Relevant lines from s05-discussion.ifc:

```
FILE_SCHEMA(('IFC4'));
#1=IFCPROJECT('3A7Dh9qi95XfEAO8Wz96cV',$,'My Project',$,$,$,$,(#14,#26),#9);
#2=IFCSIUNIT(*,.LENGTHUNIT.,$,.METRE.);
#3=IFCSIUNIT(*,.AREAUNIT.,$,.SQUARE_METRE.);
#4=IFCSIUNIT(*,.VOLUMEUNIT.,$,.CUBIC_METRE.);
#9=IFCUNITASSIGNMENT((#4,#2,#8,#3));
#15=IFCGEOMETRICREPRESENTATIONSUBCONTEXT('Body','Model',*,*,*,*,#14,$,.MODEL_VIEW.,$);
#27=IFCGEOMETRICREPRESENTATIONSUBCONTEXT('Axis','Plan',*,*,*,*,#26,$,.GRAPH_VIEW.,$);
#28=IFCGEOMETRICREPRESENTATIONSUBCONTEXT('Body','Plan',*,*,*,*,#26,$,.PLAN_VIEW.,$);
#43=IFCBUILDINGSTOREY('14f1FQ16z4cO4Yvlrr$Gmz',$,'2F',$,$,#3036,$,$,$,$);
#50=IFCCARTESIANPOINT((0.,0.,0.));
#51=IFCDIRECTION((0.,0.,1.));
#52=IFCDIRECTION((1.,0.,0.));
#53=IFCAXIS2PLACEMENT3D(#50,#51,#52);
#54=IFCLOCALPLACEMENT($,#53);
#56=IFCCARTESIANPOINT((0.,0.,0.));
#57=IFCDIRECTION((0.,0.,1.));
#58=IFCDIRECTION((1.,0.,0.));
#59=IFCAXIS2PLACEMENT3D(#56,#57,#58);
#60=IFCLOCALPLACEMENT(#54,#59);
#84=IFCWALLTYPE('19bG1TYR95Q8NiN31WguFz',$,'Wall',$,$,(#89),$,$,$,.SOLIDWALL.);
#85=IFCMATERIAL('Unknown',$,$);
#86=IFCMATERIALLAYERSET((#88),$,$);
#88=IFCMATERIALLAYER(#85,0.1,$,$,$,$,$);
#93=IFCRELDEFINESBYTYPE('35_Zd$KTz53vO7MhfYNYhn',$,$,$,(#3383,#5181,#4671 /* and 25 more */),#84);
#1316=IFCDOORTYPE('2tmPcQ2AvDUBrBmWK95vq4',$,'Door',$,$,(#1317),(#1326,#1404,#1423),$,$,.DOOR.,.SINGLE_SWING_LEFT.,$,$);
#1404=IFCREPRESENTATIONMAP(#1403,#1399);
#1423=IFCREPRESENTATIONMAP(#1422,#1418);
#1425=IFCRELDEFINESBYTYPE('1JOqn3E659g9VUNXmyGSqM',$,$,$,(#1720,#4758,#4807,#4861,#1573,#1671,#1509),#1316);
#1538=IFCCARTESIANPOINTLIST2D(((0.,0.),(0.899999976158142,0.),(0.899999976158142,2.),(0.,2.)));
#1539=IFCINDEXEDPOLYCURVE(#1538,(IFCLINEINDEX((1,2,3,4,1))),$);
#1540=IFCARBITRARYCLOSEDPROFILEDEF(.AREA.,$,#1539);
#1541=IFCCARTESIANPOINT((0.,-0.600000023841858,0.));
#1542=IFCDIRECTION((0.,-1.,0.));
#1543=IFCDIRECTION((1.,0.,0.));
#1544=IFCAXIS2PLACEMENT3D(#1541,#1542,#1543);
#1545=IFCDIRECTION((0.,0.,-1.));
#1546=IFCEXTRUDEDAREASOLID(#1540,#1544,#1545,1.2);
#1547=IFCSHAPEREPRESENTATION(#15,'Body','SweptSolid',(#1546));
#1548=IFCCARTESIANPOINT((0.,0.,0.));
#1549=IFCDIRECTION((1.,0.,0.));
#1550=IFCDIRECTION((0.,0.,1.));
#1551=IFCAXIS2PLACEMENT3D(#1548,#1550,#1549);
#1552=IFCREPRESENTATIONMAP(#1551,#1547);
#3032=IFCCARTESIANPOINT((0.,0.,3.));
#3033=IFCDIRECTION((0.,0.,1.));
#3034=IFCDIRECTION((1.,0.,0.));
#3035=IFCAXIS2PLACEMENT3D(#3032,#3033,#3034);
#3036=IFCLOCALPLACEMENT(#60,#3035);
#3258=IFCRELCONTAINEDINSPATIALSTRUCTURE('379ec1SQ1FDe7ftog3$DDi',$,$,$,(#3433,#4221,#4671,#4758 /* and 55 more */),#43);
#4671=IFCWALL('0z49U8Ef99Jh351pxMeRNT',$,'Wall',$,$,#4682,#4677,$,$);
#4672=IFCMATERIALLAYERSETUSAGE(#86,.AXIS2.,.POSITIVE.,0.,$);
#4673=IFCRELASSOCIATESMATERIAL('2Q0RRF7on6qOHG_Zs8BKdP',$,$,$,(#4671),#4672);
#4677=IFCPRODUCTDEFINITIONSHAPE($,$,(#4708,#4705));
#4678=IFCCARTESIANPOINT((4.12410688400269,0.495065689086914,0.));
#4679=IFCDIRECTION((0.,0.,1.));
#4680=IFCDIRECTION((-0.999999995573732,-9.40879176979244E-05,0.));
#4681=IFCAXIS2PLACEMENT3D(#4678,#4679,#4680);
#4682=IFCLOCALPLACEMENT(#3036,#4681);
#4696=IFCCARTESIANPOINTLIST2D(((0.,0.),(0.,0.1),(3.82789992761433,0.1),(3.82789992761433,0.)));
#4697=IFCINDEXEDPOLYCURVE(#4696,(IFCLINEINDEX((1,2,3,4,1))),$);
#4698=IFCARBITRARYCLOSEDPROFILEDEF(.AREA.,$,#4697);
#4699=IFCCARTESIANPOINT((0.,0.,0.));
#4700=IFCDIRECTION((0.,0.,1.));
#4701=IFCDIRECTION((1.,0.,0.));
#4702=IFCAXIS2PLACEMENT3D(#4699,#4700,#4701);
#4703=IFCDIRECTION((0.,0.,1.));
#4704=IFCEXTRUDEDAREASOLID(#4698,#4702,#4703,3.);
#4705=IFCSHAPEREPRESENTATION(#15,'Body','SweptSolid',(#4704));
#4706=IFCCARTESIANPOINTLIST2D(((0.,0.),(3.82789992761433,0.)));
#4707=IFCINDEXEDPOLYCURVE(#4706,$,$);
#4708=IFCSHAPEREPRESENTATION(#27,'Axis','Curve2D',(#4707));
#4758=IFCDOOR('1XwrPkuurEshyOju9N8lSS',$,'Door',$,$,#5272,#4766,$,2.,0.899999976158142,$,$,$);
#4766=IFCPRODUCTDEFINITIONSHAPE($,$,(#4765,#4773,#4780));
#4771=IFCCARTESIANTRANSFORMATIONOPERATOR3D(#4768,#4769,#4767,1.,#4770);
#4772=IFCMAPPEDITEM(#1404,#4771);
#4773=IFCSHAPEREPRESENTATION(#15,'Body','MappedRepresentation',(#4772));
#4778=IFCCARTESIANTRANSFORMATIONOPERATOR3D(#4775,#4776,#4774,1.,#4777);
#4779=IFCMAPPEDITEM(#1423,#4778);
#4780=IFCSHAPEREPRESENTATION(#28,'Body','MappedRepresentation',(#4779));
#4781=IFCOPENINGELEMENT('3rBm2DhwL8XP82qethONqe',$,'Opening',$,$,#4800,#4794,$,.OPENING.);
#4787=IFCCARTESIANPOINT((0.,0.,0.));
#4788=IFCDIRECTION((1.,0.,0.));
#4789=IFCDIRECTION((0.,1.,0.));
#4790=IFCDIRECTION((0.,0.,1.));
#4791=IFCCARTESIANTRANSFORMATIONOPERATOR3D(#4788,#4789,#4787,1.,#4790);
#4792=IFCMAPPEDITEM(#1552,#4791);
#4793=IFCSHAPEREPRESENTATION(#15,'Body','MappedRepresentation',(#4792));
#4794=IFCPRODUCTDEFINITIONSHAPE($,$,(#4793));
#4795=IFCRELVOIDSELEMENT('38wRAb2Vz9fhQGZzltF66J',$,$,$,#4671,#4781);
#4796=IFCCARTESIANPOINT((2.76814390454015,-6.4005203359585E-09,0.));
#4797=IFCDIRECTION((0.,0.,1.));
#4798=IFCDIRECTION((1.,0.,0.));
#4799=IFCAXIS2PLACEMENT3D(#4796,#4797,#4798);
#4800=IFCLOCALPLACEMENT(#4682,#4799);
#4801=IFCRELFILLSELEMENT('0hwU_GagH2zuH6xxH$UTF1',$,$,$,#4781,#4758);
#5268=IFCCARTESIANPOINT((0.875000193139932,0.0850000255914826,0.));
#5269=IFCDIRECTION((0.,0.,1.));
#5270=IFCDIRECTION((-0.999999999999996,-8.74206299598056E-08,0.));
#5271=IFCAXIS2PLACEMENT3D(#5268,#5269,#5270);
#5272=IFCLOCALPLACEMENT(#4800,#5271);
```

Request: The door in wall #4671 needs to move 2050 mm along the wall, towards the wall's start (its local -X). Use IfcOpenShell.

```python
import ifcopenshell
import ifcopenshell.api.geometry
import ifcopenshell.util.placement
import ifcopenshell.util.unit

model = ifcopenshell.open("s05-discussion.ifc")
unit_scale = ifcopenshell.util.unit.calculate_unit_scale(model)

door = model.by_guid("1XwrPkuurEshyOju9N8lSS")
opening = door.FillsVoids[0].RelatingOpeningElement
wall = opening.VoidsElements[0].RelatingBuildingElement

wall_matrix = ifcopenshell.util.placement.get_local_placement(wall.ObjectPlacement)
shift = wall_matrix[:3, 0] * -2.05 / unit_scale
before = ifcopenshell.util.placement.get_local_placement(door.ObjectPlacement)[:3, 3].copy()

# The door is placed relative to its opening, so it follows when the opening moves.
matrix = ifcopenshell.util.placement.get_local_placement(opening.ObjectPlacement)
matrix[:3, 3] += shift
ifcopenshell.api.geometry.edit_object_placement(
    model, product=opening, matrix=matrix, is_si=False, should_transform_children=True
)

after = ifcopenshell.util.placement.get_local_placement(door.ObjectPlacement)[:3, 3]
print("door moved by", (after - before).round(3) + 0.0)

model.write("s05-discussion-out.ifc")
```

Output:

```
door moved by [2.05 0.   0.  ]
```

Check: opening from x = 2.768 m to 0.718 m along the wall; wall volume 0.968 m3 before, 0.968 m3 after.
